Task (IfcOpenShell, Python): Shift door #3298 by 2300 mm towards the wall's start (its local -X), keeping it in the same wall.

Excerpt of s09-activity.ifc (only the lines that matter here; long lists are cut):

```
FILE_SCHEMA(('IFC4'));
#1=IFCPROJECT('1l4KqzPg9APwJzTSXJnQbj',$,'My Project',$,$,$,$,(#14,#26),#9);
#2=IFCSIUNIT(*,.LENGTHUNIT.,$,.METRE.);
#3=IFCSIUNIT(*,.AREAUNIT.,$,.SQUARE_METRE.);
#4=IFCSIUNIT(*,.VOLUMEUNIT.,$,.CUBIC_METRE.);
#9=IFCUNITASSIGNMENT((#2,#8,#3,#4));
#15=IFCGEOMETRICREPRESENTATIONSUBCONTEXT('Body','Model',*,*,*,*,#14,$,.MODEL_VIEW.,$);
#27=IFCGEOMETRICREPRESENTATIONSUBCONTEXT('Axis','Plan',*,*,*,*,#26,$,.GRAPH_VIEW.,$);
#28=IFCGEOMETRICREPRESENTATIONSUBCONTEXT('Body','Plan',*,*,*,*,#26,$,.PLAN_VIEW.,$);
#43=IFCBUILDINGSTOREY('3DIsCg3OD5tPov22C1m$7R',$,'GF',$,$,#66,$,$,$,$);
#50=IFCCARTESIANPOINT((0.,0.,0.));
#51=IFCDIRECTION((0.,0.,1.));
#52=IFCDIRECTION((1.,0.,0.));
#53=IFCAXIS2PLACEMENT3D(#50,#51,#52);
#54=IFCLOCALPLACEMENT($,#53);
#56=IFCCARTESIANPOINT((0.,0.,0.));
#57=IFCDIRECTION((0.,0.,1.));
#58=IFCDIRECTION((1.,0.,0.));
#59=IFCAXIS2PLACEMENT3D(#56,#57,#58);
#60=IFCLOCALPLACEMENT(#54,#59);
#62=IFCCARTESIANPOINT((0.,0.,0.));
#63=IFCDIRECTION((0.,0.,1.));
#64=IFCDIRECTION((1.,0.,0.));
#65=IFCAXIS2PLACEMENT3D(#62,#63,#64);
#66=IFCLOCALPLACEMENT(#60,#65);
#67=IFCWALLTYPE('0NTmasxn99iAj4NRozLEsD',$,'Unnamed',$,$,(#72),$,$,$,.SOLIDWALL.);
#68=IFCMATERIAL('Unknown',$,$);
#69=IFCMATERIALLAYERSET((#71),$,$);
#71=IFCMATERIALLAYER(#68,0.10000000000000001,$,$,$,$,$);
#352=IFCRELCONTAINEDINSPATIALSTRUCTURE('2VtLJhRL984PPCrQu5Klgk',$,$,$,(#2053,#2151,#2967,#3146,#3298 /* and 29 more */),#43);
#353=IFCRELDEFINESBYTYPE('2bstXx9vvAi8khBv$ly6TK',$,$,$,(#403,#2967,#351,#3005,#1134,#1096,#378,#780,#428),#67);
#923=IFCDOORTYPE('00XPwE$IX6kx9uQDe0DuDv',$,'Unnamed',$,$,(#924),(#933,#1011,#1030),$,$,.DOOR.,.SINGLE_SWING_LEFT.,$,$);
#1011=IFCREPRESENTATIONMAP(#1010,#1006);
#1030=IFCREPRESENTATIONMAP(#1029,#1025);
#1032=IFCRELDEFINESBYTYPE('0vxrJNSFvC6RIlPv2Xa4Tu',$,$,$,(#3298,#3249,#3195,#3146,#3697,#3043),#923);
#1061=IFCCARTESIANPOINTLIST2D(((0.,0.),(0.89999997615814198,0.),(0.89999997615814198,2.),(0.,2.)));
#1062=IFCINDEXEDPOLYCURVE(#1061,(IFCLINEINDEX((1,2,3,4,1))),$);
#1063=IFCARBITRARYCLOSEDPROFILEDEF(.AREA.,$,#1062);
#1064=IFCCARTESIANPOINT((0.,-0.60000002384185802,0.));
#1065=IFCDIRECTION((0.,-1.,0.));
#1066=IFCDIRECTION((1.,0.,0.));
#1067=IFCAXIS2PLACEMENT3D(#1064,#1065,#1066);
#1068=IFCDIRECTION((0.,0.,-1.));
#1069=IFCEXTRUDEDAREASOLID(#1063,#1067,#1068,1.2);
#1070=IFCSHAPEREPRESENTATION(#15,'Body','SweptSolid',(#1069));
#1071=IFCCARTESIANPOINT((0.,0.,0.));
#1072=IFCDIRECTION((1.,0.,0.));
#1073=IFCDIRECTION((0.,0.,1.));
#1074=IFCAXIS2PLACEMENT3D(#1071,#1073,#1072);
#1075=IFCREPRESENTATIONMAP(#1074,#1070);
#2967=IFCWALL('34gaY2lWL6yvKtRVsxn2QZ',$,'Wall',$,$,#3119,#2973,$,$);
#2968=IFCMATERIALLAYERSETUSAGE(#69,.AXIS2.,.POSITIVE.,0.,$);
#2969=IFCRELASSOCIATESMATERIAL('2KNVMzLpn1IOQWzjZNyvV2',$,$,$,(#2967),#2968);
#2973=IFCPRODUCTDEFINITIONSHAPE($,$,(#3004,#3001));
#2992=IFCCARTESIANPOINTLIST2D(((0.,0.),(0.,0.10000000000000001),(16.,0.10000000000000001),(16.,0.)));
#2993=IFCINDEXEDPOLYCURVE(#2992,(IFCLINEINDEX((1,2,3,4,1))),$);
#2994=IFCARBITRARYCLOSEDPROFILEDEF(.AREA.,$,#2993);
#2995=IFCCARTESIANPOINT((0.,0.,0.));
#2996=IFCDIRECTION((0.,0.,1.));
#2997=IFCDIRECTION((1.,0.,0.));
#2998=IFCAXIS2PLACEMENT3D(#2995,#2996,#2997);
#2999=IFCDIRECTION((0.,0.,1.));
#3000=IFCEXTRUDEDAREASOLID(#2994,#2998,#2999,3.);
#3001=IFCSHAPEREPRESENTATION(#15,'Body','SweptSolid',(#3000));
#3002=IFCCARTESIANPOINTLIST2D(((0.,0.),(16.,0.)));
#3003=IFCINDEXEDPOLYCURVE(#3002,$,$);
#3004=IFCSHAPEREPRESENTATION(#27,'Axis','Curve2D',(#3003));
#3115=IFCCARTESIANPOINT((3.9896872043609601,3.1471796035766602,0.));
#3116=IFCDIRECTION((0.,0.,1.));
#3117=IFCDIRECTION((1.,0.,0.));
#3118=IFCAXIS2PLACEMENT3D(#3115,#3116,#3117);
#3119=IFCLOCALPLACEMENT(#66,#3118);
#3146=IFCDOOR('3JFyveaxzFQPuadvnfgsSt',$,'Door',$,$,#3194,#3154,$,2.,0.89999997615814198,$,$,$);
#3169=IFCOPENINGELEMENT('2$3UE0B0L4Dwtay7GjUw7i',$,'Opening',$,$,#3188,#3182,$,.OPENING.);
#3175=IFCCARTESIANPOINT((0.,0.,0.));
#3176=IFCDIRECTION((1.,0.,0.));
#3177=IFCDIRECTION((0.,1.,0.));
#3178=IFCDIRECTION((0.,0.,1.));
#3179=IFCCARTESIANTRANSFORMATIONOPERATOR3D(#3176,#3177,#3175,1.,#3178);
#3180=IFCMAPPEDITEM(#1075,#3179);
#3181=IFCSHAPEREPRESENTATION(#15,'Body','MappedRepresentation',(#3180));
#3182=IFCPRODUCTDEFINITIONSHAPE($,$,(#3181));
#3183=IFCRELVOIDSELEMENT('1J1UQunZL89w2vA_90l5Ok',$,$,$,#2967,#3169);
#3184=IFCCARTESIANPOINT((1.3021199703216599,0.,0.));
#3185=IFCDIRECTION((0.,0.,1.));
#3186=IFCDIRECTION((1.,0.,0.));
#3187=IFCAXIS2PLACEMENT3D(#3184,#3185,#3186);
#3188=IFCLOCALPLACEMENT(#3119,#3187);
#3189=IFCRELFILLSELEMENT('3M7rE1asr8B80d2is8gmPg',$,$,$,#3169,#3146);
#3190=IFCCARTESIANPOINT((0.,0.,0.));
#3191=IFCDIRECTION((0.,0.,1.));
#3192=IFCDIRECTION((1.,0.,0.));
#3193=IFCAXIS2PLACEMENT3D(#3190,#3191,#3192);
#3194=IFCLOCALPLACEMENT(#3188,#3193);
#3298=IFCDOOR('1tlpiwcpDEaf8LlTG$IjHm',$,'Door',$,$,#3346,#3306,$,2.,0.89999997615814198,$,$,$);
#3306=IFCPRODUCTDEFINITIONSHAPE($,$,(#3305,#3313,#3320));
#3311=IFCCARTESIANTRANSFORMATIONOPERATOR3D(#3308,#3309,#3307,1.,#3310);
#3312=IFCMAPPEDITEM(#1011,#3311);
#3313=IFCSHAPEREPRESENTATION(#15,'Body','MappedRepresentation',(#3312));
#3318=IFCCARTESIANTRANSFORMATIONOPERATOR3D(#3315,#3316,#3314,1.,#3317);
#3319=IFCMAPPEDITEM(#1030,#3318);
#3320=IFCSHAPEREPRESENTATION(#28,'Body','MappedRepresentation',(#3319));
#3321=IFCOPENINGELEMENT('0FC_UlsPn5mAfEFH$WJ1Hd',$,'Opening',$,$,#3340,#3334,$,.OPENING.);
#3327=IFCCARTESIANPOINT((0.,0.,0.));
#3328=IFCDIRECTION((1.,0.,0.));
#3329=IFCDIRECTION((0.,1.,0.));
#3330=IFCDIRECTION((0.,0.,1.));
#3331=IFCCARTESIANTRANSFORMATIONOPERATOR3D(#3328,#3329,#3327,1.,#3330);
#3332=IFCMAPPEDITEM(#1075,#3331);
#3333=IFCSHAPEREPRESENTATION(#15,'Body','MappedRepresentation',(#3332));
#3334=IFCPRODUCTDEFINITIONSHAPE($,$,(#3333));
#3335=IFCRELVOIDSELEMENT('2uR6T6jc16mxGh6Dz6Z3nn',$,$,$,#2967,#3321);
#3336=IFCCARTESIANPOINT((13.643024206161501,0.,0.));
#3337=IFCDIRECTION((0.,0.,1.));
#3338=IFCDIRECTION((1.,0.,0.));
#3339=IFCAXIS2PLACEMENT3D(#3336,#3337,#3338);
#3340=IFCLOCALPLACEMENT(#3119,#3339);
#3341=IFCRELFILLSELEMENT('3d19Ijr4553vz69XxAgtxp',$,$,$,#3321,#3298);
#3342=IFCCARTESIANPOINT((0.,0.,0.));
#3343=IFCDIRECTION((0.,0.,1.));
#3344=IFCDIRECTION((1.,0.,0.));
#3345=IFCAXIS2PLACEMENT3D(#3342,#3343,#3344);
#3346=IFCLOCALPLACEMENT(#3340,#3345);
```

```python
import ifcopenshell
import ifcopenshell.api.geometry
import ifcopenshell.util.placement
import ifcopenshell.util.unit

model = ifcopenshell.open("s09-activity.ifc")
unit_scale = ifcopenshell.util.unit.calculate_unit_scale(model)

door = model.by_guid("1tlpiwcpDEaf8LlTG$IjHm")
opening = door.FillsVoids[0].RelatingOpeningElement
wall = opening.VoidsElements[0].RelatingBuildingElement

wall_matrix = ifcopenshell.util.placement.get_local_placement(wall.ObjectPlacement)
shift = wall_matrix[:3, 0] * -2.3 / unit_scale
before = ifcopenshell.util.placement.get_local_placement(door.ObjectPlacement)[:3, 3].copy()

# The door is placed relative to its opening, so it follows when the opening moves.
matrix = ifcopenshell.util.placement.get_local_placement(opening.ObjectPlacement)
matrix[:3, 3] += shift
ifcopenshell.api.geometry.edit_object_placement(
    model, product=opening, matrix=matrix, is_si=False, should_transform_children=True
)

after = ifcopenshell.util.placement.get_local_placement(door.ObjectPlacement)[:3, 3]
print("door moved by", (after - before).round(3) + 0.0)

model.write("s09-activity_v2.ifc")
```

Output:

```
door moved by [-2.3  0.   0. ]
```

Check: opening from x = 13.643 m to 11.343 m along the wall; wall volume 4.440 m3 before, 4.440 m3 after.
